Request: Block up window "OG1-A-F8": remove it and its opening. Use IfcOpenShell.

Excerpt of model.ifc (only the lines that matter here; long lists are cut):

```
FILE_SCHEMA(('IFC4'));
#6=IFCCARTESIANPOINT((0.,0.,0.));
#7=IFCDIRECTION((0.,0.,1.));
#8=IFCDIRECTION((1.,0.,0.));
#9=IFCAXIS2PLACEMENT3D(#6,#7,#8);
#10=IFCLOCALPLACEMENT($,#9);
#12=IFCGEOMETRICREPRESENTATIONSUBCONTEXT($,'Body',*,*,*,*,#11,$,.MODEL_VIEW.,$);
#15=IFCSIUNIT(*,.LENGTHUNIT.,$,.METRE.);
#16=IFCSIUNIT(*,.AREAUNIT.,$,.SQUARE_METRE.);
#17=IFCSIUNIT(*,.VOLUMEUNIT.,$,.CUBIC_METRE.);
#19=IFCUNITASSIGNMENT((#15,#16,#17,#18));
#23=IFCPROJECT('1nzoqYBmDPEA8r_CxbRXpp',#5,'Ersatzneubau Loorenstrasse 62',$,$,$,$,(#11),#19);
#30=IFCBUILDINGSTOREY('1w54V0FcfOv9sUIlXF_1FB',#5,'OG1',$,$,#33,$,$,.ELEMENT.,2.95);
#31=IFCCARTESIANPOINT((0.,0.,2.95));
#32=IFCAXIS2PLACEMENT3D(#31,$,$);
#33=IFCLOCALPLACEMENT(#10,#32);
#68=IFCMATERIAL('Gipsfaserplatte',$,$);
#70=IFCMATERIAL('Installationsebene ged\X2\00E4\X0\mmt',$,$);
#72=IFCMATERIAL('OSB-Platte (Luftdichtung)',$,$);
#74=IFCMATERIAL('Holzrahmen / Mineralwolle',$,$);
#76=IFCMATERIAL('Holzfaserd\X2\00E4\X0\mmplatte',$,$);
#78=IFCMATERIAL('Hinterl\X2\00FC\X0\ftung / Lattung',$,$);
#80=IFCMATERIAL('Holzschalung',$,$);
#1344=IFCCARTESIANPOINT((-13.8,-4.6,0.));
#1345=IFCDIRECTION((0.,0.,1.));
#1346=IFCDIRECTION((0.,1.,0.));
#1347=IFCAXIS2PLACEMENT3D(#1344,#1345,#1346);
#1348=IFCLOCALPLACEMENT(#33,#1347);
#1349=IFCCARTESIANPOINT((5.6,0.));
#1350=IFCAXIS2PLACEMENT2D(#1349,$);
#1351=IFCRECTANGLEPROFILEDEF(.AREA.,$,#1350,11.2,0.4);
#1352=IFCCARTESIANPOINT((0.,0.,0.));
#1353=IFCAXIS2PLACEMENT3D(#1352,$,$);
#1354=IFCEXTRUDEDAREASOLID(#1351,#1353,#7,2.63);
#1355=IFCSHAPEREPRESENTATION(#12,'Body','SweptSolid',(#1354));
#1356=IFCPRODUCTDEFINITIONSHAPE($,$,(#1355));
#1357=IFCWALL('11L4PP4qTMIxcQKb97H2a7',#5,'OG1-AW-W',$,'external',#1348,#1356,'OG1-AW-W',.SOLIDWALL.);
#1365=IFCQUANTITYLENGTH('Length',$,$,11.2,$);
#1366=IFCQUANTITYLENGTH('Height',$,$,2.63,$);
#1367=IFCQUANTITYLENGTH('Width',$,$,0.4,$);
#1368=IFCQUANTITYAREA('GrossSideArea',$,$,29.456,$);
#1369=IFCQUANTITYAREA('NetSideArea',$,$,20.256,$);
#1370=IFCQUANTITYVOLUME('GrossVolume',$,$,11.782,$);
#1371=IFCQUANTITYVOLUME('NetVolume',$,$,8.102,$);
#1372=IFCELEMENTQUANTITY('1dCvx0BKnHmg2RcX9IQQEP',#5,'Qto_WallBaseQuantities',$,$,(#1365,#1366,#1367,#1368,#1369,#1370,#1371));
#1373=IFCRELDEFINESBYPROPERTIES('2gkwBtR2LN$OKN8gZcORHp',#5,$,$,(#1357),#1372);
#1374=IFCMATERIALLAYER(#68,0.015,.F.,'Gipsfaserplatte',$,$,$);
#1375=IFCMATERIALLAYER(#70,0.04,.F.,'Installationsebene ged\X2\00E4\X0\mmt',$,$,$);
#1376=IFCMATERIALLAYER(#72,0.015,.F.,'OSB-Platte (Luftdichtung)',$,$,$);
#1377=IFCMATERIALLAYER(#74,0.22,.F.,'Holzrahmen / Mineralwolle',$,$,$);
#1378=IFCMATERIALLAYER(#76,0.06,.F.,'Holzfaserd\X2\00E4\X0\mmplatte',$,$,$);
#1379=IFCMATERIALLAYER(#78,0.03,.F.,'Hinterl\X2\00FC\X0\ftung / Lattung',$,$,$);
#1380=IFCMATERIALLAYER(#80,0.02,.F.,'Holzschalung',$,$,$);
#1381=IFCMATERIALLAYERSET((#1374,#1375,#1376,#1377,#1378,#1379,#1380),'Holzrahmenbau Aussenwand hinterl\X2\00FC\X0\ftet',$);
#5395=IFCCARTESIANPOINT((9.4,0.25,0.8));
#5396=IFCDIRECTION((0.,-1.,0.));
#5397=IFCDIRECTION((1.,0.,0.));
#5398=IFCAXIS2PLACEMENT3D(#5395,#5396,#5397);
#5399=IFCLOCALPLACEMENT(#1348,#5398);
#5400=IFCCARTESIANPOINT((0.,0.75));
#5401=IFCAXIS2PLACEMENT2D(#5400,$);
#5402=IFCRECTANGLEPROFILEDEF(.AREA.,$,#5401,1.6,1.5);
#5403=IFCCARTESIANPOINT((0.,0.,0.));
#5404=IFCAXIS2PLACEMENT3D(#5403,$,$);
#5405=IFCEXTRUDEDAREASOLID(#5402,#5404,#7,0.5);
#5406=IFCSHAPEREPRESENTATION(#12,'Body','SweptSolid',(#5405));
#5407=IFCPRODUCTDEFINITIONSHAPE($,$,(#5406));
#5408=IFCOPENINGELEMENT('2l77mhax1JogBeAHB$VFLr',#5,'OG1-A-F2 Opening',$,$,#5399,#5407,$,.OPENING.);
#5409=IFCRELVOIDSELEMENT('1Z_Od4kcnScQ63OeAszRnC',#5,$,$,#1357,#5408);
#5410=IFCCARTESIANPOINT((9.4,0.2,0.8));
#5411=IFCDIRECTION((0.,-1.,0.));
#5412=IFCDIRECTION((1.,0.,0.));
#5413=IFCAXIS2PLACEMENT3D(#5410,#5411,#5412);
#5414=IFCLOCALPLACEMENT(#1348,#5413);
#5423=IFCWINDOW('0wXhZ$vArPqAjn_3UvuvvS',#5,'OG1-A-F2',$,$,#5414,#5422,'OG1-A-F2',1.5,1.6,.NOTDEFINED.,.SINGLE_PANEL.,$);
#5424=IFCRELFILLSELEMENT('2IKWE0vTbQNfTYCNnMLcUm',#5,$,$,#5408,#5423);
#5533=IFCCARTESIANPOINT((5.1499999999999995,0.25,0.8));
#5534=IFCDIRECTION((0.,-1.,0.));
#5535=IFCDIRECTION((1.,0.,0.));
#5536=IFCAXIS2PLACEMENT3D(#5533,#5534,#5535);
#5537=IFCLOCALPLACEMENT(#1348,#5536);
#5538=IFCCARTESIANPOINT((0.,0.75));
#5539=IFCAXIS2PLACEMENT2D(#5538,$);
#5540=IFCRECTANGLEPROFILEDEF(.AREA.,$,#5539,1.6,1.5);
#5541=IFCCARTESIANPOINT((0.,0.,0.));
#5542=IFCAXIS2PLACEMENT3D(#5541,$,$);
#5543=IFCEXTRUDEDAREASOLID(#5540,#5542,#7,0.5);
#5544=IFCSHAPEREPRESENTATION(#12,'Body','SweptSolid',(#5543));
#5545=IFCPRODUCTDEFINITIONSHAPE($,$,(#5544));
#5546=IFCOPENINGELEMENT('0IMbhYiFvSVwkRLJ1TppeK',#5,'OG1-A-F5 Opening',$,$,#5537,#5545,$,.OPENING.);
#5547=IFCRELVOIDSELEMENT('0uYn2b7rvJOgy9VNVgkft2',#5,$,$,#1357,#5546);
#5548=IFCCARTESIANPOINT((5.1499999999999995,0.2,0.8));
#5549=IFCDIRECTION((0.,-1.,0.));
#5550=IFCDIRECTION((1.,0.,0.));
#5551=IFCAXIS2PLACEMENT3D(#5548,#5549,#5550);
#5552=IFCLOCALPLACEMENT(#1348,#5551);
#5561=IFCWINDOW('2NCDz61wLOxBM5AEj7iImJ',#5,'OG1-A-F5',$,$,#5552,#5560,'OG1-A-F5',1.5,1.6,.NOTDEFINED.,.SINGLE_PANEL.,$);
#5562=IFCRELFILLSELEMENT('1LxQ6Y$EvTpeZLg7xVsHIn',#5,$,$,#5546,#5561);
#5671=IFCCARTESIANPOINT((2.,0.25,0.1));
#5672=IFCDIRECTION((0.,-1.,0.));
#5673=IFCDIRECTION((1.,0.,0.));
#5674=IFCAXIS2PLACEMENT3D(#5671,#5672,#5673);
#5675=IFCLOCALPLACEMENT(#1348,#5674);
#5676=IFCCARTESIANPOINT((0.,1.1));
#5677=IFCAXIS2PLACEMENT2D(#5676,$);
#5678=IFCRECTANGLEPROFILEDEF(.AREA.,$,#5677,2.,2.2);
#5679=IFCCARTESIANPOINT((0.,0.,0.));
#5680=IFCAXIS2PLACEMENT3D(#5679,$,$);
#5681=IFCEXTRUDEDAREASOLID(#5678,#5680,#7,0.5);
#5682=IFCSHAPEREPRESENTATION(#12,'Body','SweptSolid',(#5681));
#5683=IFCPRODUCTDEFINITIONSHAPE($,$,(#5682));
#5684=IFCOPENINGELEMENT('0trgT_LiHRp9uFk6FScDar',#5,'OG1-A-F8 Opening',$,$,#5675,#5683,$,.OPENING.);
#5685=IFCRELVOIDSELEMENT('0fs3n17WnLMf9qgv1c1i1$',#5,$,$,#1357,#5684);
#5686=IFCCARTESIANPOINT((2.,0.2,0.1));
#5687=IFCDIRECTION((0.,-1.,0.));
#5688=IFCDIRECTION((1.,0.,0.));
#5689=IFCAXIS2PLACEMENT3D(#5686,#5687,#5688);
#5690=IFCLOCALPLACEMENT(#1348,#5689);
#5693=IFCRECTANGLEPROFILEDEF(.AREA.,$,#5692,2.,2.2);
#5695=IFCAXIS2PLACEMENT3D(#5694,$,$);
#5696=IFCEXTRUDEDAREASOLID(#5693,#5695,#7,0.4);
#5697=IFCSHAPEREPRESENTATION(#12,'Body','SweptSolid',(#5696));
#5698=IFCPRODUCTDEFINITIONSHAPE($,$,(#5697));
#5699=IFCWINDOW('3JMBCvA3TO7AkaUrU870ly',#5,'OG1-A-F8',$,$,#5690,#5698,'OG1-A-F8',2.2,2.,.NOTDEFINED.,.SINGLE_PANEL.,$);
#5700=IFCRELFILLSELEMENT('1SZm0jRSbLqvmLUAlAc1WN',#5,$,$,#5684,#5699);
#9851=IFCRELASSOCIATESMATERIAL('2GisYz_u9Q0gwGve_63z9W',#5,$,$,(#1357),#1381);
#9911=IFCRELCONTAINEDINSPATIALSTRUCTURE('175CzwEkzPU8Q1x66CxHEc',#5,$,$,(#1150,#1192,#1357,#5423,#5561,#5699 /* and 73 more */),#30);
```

```python
import ifcopenshell
import ifcopenshell.api.feature
import ifcopenshell.api.pset
import ifcopenshell.api.root
import ifcopenshell.geom
import ifcopenshell.util.element
import ifcopenshell.util.shape
import ifcopenshell.util.unit

model = ifcopenshell.open("model.ifc")
area_scale = ifcopenshell.util.unit.calculate_unit_scale(model, "AREAUNIT")
volume_scale = ifcopenshell.util.unit.calculate_unit_scale(model, "VOLUMEUNIT")
settings = ifcopenshell.geom.settings()


def volume(element):
    """Net volume in cubic metres, openings subtracted."""
    shape = ifcopenshell.geom.create_shape(settings, element)
    return ifcopenshell.util.shape.get_volume(shape.geometry)


window = model.by_guid("3JMBCvA3TO7AkaUrU870ly")
opening = window.FillsVoids[0].RelatingOpeningElement
wall = opening.VoidsElements[0].RelatingBuildingElement
before = volume(wall)

ifcopenshell.api.root.remove_product(model, product=window)
ifcopenshell.api.feature.remove_feature(model, feature=opening)

after = volume(wall)
thickness = 0.4  # wall thickness in metres

# Update the wall's stored quantities.
qto = model.by_id(ifcopenshell.util.element.get_pset(wall, "Qto_WallBaseQuantities", should_inherit=False)["id"])
ifcopenshell.api.pset.edit_qto(model, qto=qto, properties={
    "NetSideArea": after / thickness / area_scale,
    "NetVolume": after / volume_scale,
})

print(f"wall volume {before:.3f} -> {after:.3f} m3")

model.write("model_v2.ifc")
```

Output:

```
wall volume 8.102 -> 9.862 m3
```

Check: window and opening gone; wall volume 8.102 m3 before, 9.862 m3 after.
